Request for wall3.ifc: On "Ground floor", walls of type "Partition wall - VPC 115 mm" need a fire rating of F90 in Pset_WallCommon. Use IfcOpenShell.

First a look at what the model holds.

```python
import ifcopenshell
import ifcopenshell.util.element

model = ifcopenshell.open("wall3.ifc")
print(model.schema)
storey = next(s for s in model.by_type("IfcBuildingStorey") if s.Name == "Ground floor")
walls = [e for e in ifcopenshell.util.element.get_decomposition(storey) if e.is_a("IfcWall")]
seen = {}
for e in walls:
    element_type = ifcopenshell.util.element.get_type(e)
    key = (element_type.Name if element_type != e and element_type else None, ifcopenshell.util.element.get_pset(e, "Pset_WallCommon", "FireRating"))
    seen[key] = seen.get(key, 0) + 1
for (name, value), count in sorted(seen.items(), key=str):
    print(count, "x", name, "|", value)
```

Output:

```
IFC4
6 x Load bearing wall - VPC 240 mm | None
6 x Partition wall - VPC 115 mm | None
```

```python
import ifcopenshell
import ifcopenshell.api.pset
import ifcopenshell.util.element

model = ifcopenshell.open("wall3.ifc")

storey = next(s for s in model.by_type("IfcBuildingStorey") if s.Name == "Ground floor")
walls = [e for e in ifcopenshell.util.element.get_decomposition(storey) if e.is_a("IfcWall")]

count = 0
for e in walls:
    element_type = ifcopenshell.util.element.get_type(e)
    if element_type in (None, e) or element_type.Name != "Partition wall - VPC 115 mm":
        continue
    # add_pset returns the element's existing set when there is one.
    pset = ifcopenshell.api.pset.add_pset(model, product=e, name="Pset_WallCommon")
    ifcopenshell.api.pset.edit_pset(model, pset=pset, properties={"FireRating": "F90"})
    count += 1

print(count, "walls updated")

model.write("wall3_edited.ifc")
```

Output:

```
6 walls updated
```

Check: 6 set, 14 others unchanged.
